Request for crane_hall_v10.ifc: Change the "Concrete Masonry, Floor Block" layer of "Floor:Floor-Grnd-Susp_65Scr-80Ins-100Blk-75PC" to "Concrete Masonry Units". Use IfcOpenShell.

First a look at what the model holds.

```python
import ifcopenshell
import ifcopenshell.util.element

model = ifcopenshell.open("crane_hall_v10.ifc")
print(model.schema)
for layer_set in model.by_type("IfcMaterialLayerSet"):
    if layer_set.LayerSetName == "Floor:Floor-Grnd-Susp_65Scr-80Ins-100Blk-75PC":
        for layer in layer_set.MaterialLayers:
            print(layer.id(), layer.Material and layer.Material.Name, layer.LayerThickness, sep=" | ")
        print(len(ifcopenshell.util.element.get_elements_by_material(model, layer_set)), "elements and types use it")
print(sorted(m.Name for m in model.by_type("IfcMaterial") if m.Name)[:60])
```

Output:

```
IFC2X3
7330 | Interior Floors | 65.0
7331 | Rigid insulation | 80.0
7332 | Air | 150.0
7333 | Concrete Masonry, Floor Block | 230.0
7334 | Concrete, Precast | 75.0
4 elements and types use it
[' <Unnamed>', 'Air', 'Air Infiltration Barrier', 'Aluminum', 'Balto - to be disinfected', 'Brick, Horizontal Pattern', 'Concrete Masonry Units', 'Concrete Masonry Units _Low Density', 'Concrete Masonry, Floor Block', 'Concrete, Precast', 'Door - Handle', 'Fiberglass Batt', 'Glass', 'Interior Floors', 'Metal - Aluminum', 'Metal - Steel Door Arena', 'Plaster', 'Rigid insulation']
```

```python
import ifcopenshell
import ifcopenshell.api.material

model = ifcopenshell.open("crane_hall_v10.ifc")

layer_set = next(s for s in model.by_type("IfcMaterialLayerSet") if s.LayerSetName == "Floor:Floor-Grnd-Susp_65Scr-80Ins-100Blk-75PC")
layer = next(l for l in layer_set.MaterialLayers if l.Material and l.Material.Name == "Concrete Masonry, Floor Block")
material = next(m for m in model.by_type("IfcMaterial") if m.Name == "Concrete Masonry Units")

# Point this one layer at the other material; renaming the old one would change it everywhere.
ifcopenshell.api.material.edit_layer(model, layer=layer, attributes={}, material=material)

print([l.Material.Name if l.Material else None for l in layer_set.MaterialLayers])

model.write("crane_hall_v10-out.ifc")
```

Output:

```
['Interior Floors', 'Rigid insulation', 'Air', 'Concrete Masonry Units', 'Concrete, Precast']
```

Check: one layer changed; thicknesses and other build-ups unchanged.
